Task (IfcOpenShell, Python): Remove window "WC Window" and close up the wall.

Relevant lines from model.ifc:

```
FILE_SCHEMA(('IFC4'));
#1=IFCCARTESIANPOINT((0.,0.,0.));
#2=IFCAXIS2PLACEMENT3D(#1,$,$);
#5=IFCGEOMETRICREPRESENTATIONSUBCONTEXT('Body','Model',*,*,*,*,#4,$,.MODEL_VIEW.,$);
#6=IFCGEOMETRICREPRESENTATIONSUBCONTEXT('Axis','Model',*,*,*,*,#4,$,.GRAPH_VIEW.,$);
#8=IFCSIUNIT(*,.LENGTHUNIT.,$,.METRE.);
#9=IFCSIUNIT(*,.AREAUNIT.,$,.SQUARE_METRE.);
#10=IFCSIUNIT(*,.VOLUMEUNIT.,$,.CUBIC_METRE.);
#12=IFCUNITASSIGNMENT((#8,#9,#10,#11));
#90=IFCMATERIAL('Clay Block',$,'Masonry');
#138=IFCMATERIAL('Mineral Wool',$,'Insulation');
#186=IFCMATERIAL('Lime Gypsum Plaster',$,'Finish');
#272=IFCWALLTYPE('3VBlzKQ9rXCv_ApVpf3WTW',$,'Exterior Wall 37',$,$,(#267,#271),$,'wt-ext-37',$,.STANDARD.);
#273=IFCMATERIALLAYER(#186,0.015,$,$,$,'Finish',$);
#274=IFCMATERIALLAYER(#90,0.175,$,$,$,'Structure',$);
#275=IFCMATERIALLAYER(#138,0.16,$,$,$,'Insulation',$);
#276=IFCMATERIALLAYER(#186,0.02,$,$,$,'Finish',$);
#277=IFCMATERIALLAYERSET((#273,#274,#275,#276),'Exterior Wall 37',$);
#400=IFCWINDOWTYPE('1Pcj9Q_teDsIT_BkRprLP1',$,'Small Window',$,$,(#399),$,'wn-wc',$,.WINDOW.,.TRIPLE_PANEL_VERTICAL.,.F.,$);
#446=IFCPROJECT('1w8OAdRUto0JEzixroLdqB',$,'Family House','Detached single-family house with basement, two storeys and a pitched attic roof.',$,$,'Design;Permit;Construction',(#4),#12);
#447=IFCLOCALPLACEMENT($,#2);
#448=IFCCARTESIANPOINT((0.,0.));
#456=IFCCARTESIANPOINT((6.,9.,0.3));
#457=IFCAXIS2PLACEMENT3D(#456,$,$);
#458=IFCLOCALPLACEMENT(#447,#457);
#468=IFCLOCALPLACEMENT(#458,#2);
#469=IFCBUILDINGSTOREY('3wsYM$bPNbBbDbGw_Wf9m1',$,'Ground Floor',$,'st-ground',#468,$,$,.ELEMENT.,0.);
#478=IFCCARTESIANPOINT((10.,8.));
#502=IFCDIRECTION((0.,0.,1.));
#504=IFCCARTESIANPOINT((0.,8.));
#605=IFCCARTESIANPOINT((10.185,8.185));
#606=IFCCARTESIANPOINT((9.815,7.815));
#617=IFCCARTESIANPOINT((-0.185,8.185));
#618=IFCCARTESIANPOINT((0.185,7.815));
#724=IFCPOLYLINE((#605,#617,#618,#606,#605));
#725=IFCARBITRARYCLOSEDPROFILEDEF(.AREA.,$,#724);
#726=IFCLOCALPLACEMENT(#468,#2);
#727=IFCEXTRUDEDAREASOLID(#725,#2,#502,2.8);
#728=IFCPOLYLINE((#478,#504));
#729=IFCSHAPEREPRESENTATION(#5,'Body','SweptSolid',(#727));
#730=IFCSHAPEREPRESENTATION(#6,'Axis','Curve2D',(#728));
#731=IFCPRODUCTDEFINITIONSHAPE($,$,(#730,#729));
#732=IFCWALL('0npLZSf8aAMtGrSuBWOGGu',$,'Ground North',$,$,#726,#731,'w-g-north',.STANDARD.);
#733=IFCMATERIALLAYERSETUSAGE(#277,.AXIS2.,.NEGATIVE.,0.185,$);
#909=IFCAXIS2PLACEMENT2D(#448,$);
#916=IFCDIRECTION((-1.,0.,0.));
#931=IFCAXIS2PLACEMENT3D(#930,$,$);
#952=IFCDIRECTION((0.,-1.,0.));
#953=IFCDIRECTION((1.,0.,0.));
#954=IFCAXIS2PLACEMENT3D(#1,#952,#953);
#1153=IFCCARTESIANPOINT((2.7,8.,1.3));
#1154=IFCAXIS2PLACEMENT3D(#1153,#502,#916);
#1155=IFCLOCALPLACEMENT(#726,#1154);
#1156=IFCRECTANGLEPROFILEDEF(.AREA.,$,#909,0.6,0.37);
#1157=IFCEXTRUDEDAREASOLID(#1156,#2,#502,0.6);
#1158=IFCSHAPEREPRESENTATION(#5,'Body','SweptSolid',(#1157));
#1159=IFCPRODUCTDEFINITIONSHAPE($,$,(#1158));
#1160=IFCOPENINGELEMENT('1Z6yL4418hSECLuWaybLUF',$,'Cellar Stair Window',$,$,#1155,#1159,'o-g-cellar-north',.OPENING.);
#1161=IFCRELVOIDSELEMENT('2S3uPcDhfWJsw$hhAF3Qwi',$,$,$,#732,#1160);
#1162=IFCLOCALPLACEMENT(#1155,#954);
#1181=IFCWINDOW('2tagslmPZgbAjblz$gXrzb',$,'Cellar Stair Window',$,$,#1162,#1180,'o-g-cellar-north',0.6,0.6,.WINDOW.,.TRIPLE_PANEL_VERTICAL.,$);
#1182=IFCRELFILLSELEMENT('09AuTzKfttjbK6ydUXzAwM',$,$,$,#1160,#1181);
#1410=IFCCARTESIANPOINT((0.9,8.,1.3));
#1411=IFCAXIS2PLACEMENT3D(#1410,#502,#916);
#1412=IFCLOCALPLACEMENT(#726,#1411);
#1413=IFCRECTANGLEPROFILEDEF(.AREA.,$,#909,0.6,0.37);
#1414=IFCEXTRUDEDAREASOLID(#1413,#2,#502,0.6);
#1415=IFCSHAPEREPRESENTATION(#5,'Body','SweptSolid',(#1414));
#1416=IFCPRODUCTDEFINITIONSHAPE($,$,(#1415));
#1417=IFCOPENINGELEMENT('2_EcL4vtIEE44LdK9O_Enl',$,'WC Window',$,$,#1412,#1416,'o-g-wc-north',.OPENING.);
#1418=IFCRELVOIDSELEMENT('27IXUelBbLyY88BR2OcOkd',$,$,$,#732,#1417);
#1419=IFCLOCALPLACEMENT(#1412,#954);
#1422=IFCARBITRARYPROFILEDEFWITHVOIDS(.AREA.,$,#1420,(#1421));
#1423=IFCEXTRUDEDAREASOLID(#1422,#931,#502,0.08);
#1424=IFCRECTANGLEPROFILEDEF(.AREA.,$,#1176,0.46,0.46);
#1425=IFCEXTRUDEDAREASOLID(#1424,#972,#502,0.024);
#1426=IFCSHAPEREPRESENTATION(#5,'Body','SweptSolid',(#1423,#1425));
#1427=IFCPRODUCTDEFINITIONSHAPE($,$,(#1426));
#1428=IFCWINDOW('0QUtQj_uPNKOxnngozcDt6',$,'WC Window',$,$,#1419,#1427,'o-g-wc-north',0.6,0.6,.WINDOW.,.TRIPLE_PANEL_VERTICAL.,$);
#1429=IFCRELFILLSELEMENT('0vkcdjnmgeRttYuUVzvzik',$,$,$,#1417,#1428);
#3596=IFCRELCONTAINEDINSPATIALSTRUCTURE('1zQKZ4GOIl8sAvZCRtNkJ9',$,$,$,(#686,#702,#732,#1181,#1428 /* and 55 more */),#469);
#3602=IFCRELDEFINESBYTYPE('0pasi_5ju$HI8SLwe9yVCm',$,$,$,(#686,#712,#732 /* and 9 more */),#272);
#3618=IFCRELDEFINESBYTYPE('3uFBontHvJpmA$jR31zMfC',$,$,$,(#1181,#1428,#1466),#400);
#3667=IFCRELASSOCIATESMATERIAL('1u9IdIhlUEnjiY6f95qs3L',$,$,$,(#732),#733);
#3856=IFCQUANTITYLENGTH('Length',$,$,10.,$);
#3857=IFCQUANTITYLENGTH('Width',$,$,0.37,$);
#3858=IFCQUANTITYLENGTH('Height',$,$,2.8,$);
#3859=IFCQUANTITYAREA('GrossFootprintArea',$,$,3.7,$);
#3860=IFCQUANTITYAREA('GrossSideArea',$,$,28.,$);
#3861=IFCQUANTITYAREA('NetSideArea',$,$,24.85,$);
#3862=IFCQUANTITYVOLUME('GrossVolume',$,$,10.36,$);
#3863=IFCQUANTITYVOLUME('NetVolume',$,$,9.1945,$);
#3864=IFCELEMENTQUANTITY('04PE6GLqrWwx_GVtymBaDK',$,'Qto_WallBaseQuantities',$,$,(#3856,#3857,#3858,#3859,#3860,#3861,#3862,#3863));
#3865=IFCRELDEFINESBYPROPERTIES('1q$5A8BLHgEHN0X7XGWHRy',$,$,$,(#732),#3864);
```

```python
import ifcopenshell
import ifcopenshell.api.feature
import ifcopenshell.api.pset
import ifcopenshell.api.root
import ifcopenshell.geom
import ifcopenshell.util.element
import ifcopenshell.util.shape
import ifcopenshell.util.unit

model = ifcopenshell.open("model.ifc")
area_scale = ifcopenshell.util.unit.calculate_unit_scale(model, "AREAUNIT")
volume_scale = ifcopenshell.util.unit.calculate_unit_scale(model, "VOLUMEUNIT")
settings = ifcopenshell.geom.settings()


def volume(element):
    """Net volume in cubic metres, openings subtracted."""
    shape = ifcopenshell.geom.create_shape(settings, element)
    return ifcopenshell.util.shape.get_volume(shape.geometry)


window = model.by_id(1428)
opening = window.FillsVoids[0].RelatingOpeningElement
wall = opening.VoidsElements[0].RelatingBuildingElement
before = volume(wall)

ifcopenshell.api.root.remove_product(model, product=window)
ifcopenshell.api.feature.remove_feature(model, feature=opening)

after = volume(wall)
thickness = 0.37  # wall thickness in metres

# Update the wall's stored quantities.
qto = model.by_id(ifcopenshell.util.element.get_pset(wall, "Qto_WallBaseQuantities", should_inherit=False)["id"])
ifcopenshell.api.pset.edit_qto(model, qto=qto, properties={
    "NetSideArea": after / thickness / area_scale,
    "NetVolume": after / volume_scale,
})

print(f"wall volume {before:.3f} -> {after:.3f} m3")

model.write("model_v2.ifc")
```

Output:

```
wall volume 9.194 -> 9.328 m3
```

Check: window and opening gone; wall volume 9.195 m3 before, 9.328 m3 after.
